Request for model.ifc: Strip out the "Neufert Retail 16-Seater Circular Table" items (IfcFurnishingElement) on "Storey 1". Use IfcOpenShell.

First a look at what the model holds.

```python
import ifcopenshell
import ifcopenshell.util.element

model = ifcopenshell.open("model.ifc")
print(model.schema)
storey = next(s for s in model.by_type("IfcBuildingStorey") if s.Name == "Storey 1")
furniture = [e for e in ifcopenshell.util.element.get_decomposition(storey) if e.is_a("IfcFurnishingElement")]
seen = {}
for e in furniture:
    element_type = ifcopenshell.util.element.get_type(e)
    name = element_type.Name if element_type not in (None, e) else None
    seen[name] = seen.get(name, 0) + 1
for name, count in sorted(seen.items(), key=str):
    print(count, "x", name)
```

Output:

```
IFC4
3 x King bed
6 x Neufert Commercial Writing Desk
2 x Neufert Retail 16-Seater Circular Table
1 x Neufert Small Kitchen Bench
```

```python
import ifcopenshell
import ifcopenshell.api.root
import ifcopenshell.util.element

model = ifcopenshell.open("model.ifc")

storey = next(s for s in model.by_type("IfcBuildingStorey") if s.Name == "Storey 1")
furniture = [e for e in ifcopenshell.util.element.get_decomposition(storey) if e.is_a("IfcFurnishingElement")]
targets = [e for e in furniture if (t := ifcopenshell.util.element.get_type(e)) not in (None, e) and t.Name == "Neufert Retail 16-Seater Circular Table"]

for e in targets:
    ifcopenshell.api.root.remove_product(model, product=e)
print(len(targets), "removed")

model.write("model_edited.ifc")
```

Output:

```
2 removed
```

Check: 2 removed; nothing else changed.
